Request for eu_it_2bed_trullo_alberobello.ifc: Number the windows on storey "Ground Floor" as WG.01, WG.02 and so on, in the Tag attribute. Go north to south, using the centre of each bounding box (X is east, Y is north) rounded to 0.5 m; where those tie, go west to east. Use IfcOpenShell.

First a look at what the model holds.

```python
import ifcopenshell
import ifcopenshell.util.element
import ifcopenshell.util.placement

model = ifcopenshell.open("eu_it_2bed_trullo_alberobello.ifc")
print(model.schema)
storey = next(s for s in model.by_type("IfcBuildingStorey") if s.Name == "Ground Floor")
windows = [e for e in ifcopenshell.util.element.get_decomposition(storey) if e.is_a("IfcWindow")]
for e in sorted(windows, key=lambda e: e.id()):
    origin = ifcopenshell.util.placement.get_local_placement(e.ObjectPlacement)[:3, 3]
    print(e.id(), e.Tag, e.Name, origin.round(2) + 0.0, sep=" | ")
```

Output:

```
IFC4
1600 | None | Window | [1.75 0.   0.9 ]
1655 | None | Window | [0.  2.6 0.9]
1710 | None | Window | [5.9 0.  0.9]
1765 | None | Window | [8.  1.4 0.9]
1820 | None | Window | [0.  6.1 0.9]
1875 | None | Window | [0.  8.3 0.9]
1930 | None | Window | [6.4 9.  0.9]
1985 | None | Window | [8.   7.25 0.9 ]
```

```python
import ifcopenshell
import ifcopenshell.geom
import ifcopenshell.util.element
import ifcopenshell.util.shape

model = ifcopenshell.open("eu_it_2bed_trullo_alberobello.ifc")
settings = ifcopenshell.geom.settings()
settings.set("use-world-coords", True)


def centre(element):
    shape = ifcopenshell.geom.create_shape(settings, element)
    return ifcopenshell.util.shape.get_bbox_centroid(shape.geometry)


storey = next(s for s in model.by_type("IfcBuildingStorey") if s.Name == "Ground Floor")
windows = [e for e in ifcopenshell.util.element.get_decomposition(storey) if e.is_a("IfcWindow")]

# Insertion points can sit at a corner or the storey origin, so sort by the geometry (in metres).
centres = {e: centre(e) for e in windows}
windows.sort(key=lambda e: (-round(centres[e][1] / 0.5), centres[e][0]))

for i, e in enumerate(windows, start=1):
    number = f"WG.{i:02d}"
    e.Tag = number
    print(e.id(), number)

model.write("eu_it_2bed_trullo_alberobello_rev.ifc")
```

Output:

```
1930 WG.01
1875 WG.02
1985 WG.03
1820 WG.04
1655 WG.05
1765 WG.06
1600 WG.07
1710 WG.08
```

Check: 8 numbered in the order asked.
